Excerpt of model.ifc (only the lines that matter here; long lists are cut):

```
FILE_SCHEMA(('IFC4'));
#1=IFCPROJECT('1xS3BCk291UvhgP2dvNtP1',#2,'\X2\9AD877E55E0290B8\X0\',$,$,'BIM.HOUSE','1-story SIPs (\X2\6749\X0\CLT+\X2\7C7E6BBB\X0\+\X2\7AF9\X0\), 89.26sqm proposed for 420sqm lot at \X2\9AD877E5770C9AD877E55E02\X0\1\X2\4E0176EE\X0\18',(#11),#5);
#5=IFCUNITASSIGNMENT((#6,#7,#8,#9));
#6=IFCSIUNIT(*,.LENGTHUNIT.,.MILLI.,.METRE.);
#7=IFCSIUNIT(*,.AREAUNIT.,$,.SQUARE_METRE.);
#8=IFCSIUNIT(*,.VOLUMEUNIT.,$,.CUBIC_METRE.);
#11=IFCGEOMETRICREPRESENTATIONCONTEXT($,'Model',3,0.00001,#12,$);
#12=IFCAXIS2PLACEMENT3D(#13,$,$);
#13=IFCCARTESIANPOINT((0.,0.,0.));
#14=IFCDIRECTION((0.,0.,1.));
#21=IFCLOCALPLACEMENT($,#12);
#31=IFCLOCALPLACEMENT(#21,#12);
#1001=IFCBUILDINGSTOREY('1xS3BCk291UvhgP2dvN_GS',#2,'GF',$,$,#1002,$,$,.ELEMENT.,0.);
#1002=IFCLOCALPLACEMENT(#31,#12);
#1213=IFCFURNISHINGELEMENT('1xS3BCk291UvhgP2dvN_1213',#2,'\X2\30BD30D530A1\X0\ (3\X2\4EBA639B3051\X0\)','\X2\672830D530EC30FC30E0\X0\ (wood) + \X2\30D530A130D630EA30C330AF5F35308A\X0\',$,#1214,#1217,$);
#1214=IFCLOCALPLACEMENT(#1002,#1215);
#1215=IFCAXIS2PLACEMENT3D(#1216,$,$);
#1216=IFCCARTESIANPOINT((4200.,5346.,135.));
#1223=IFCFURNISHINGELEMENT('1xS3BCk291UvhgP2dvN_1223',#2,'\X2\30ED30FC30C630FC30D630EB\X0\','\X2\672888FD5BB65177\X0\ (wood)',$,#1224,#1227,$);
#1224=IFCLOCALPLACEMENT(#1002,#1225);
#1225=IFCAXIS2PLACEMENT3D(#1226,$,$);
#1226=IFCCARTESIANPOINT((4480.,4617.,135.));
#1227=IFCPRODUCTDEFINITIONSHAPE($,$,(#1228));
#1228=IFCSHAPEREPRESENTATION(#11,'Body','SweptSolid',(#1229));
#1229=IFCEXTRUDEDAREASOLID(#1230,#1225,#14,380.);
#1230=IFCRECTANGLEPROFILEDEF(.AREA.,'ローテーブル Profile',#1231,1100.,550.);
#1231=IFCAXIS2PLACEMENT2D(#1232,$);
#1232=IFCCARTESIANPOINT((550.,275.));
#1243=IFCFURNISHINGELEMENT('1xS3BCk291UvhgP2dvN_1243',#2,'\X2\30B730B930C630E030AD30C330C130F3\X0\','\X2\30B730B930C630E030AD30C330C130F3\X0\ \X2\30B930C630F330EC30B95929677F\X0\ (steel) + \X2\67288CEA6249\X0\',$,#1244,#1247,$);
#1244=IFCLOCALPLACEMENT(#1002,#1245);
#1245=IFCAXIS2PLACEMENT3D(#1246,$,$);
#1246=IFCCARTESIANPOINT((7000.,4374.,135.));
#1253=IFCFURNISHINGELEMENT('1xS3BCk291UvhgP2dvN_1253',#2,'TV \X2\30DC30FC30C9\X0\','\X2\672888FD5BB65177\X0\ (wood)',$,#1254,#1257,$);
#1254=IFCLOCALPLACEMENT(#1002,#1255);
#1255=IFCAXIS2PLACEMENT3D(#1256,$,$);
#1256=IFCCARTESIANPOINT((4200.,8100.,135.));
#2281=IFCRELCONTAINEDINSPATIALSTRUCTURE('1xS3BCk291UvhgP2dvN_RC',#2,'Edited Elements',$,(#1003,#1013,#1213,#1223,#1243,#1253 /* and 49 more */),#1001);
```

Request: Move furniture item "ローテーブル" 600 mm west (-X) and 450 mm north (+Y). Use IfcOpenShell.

```python
import ifcopenshell
import ifcopenshell.api.geometry
import ifcopenshell.util.placement
import ifcopenshell.util.unit

model = ifcopenshell.open("model.ifc")
unit_scale = ifcopenshell.util.unit.calculate_unit_scale(model)

item = model.by_guid("1xS3BCk291UvhgP2dvN_1223")
matrix = ifcopenshell.util.placement.get_local_placement(item.ObjectPlacement)
matrix[0, 3] -= 0.6 / unit_scale
matrix[1, 3] += 0.45 / unit_scale
ifcopenshell.api.geometry.edit_object_placement(model, product=item, matrix=matrix, is_si=False)

print(ifcopenshell.util.placement.get_local_placement(item.ObjectPlacement).round(3) + 0.0)

model.write("model_rev.ifc")
```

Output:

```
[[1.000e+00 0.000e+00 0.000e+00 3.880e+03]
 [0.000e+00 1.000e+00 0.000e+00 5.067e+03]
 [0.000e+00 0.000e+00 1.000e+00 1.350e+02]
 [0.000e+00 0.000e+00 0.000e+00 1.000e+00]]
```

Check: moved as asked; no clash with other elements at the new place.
